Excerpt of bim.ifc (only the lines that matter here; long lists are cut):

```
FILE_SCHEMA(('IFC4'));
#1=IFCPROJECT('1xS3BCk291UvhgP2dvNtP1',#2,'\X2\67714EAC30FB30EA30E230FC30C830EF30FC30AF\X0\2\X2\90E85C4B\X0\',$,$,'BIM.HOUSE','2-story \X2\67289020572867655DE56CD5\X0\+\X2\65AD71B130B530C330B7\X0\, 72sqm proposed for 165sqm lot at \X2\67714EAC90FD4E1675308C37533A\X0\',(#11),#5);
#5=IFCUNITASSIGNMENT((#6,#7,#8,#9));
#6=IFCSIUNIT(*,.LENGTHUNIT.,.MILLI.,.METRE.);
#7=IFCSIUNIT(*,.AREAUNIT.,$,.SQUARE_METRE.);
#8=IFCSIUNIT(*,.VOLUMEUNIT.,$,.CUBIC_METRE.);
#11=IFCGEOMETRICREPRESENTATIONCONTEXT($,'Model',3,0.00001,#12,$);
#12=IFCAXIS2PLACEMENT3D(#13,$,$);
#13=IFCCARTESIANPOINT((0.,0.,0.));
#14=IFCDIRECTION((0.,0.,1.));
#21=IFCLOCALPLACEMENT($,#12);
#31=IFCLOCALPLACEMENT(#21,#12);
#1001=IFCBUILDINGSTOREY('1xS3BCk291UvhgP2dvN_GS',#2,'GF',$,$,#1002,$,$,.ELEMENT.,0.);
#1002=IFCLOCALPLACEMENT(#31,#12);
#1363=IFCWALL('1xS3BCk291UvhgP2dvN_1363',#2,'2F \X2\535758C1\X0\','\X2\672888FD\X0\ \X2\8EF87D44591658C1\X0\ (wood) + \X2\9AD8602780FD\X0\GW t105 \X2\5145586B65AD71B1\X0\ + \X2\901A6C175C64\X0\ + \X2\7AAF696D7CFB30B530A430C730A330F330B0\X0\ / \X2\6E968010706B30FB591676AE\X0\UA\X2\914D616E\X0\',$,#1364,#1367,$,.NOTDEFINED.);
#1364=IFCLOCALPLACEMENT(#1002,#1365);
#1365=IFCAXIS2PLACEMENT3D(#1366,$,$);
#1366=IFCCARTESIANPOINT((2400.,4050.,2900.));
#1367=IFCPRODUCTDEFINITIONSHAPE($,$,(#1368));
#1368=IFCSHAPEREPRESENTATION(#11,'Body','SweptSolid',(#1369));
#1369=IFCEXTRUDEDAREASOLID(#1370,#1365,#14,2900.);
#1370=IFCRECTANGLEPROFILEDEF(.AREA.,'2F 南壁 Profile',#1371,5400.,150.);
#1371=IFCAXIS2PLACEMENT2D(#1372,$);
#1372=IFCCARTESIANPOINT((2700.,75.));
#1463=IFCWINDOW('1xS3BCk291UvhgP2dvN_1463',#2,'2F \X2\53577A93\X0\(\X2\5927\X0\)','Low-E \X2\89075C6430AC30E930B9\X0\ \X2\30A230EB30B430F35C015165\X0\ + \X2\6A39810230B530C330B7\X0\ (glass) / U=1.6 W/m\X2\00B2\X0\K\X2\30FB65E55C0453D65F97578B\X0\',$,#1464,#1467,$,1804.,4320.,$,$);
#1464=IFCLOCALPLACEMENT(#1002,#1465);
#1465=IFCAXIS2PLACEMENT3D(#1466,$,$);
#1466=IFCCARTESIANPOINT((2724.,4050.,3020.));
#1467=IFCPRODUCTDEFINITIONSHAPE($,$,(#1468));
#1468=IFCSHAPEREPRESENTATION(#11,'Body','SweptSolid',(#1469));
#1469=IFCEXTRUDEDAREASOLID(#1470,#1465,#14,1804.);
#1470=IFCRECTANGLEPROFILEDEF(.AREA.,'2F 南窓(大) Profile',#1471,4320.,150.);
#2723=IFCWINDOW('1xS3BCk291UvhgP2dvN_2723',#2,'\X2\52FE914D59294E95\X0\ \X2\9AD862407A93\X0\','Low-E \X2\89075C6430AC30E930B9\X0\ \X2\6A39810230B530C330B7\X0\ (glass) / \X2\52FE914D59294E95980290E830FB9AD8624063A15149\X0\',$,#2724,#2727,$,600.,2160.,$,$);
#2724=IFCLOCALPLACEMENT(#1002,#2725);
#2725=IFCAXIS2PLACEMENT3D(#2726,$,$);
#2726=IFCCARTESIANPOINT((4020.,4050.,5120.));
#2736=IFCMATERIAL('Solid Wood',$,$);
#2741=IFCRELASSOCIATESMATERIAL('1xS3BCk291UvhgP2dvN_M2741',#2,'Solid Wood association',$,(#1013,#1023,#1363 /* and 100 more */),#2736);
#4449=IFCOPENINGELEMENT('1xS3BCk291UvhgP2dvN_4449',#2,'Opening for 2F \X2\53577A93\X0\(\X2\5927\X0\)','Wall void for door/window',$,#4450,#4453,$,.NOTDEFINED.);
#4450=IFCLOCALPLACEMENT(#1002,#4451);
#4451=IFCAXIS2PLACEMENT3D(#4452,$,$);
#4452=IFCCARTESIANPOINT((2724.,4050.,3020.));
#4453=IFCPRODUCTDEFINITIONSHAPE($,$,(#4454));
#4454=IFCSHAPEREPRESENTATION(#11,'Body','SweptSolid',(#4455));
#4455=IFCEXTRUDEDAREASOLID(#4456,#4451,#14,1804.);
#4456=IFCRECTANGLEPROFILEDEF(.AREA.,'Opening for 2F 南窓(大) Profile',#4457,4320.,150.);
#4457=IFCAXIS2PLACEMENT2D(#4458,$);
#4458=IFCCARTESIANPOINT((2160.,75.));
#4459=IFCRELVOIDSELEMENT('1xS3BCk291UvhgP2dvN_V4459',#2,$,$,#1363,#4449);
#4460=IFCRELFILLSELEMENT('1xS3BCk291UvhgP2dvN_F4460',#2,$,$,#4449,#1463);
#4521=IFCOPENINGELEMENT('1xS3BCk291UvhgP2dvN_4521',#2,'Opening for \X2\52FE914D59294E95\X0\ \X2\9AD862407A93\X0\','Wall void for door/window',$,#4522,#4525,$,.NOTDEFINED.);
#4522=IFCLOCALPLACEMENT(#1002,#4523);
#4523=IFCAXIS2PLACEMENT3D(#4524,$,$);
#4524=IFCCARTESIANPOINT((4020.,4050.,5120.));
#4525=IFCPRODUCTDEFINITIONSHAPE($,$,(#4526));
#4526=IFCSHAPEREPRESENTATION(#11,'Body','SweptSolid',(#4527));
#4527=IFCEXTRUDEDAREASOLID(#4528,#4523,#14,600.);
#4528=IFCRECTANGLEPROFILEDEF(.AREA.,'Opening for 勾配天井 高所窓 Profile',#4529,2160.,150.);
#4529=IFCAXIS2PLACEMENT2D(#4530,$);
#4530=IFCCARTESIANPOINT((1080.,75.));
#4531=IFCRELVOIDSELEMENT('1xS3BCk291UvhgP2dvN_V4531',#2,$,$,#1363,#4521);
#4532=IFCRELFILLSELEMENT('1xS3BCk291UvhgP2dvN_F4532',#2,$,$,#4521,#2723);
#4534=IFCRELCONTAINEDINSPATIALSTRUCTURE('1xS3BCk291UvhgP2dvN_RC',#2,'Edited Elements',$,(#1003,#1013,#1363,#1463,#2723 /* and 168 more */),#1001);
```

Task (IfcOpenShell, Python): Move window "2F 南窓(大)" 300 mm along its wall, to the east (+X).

```python
import ifcopenshell
import ifcopenshell.api.geometry
import ifcopenshell.util.placement

model = ifcopenshell.open("bim.ifc")

window = model.by_guid("1xS3BCk291UvhgP2dvN_1463")
opening = window.FillsVoids[0].RelatingOpeningElement
wall = opening.VoidsElements[0].RelatingBuildingElement

wall_matrix = ifcopenshell.util.placement.get_local_placement(wall.ObjectPlacement)
shift = wall_matrix[:3, 0] * 300.0
before = ifcopenshell.util.placement.get_local_placement(window.ObjectPlacement)[:3, 3].copy()

# The window is not placed relative to its opening, so move both.
for product in (opening, window):
    matrix = ifcopenshell.util.placement.get_local_placement(product.ObjectPlacement)
    matrix[:3, 3] += shift
    ifcopenshell.api.geometry.edit_object_placement(model, product=product, matrix=matrix, is_si=False)

after = ifcopenshell.util.placement.get_local_placement(window.ObjectPlacement)[:3, 3]
print("window moved by", (after - before).round(3) + 0.0)

model.write("bim_edited.ifc")
```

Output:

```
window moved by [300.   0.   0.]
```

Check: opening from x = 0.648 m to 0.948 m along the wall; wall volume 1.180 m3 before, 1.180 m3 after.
